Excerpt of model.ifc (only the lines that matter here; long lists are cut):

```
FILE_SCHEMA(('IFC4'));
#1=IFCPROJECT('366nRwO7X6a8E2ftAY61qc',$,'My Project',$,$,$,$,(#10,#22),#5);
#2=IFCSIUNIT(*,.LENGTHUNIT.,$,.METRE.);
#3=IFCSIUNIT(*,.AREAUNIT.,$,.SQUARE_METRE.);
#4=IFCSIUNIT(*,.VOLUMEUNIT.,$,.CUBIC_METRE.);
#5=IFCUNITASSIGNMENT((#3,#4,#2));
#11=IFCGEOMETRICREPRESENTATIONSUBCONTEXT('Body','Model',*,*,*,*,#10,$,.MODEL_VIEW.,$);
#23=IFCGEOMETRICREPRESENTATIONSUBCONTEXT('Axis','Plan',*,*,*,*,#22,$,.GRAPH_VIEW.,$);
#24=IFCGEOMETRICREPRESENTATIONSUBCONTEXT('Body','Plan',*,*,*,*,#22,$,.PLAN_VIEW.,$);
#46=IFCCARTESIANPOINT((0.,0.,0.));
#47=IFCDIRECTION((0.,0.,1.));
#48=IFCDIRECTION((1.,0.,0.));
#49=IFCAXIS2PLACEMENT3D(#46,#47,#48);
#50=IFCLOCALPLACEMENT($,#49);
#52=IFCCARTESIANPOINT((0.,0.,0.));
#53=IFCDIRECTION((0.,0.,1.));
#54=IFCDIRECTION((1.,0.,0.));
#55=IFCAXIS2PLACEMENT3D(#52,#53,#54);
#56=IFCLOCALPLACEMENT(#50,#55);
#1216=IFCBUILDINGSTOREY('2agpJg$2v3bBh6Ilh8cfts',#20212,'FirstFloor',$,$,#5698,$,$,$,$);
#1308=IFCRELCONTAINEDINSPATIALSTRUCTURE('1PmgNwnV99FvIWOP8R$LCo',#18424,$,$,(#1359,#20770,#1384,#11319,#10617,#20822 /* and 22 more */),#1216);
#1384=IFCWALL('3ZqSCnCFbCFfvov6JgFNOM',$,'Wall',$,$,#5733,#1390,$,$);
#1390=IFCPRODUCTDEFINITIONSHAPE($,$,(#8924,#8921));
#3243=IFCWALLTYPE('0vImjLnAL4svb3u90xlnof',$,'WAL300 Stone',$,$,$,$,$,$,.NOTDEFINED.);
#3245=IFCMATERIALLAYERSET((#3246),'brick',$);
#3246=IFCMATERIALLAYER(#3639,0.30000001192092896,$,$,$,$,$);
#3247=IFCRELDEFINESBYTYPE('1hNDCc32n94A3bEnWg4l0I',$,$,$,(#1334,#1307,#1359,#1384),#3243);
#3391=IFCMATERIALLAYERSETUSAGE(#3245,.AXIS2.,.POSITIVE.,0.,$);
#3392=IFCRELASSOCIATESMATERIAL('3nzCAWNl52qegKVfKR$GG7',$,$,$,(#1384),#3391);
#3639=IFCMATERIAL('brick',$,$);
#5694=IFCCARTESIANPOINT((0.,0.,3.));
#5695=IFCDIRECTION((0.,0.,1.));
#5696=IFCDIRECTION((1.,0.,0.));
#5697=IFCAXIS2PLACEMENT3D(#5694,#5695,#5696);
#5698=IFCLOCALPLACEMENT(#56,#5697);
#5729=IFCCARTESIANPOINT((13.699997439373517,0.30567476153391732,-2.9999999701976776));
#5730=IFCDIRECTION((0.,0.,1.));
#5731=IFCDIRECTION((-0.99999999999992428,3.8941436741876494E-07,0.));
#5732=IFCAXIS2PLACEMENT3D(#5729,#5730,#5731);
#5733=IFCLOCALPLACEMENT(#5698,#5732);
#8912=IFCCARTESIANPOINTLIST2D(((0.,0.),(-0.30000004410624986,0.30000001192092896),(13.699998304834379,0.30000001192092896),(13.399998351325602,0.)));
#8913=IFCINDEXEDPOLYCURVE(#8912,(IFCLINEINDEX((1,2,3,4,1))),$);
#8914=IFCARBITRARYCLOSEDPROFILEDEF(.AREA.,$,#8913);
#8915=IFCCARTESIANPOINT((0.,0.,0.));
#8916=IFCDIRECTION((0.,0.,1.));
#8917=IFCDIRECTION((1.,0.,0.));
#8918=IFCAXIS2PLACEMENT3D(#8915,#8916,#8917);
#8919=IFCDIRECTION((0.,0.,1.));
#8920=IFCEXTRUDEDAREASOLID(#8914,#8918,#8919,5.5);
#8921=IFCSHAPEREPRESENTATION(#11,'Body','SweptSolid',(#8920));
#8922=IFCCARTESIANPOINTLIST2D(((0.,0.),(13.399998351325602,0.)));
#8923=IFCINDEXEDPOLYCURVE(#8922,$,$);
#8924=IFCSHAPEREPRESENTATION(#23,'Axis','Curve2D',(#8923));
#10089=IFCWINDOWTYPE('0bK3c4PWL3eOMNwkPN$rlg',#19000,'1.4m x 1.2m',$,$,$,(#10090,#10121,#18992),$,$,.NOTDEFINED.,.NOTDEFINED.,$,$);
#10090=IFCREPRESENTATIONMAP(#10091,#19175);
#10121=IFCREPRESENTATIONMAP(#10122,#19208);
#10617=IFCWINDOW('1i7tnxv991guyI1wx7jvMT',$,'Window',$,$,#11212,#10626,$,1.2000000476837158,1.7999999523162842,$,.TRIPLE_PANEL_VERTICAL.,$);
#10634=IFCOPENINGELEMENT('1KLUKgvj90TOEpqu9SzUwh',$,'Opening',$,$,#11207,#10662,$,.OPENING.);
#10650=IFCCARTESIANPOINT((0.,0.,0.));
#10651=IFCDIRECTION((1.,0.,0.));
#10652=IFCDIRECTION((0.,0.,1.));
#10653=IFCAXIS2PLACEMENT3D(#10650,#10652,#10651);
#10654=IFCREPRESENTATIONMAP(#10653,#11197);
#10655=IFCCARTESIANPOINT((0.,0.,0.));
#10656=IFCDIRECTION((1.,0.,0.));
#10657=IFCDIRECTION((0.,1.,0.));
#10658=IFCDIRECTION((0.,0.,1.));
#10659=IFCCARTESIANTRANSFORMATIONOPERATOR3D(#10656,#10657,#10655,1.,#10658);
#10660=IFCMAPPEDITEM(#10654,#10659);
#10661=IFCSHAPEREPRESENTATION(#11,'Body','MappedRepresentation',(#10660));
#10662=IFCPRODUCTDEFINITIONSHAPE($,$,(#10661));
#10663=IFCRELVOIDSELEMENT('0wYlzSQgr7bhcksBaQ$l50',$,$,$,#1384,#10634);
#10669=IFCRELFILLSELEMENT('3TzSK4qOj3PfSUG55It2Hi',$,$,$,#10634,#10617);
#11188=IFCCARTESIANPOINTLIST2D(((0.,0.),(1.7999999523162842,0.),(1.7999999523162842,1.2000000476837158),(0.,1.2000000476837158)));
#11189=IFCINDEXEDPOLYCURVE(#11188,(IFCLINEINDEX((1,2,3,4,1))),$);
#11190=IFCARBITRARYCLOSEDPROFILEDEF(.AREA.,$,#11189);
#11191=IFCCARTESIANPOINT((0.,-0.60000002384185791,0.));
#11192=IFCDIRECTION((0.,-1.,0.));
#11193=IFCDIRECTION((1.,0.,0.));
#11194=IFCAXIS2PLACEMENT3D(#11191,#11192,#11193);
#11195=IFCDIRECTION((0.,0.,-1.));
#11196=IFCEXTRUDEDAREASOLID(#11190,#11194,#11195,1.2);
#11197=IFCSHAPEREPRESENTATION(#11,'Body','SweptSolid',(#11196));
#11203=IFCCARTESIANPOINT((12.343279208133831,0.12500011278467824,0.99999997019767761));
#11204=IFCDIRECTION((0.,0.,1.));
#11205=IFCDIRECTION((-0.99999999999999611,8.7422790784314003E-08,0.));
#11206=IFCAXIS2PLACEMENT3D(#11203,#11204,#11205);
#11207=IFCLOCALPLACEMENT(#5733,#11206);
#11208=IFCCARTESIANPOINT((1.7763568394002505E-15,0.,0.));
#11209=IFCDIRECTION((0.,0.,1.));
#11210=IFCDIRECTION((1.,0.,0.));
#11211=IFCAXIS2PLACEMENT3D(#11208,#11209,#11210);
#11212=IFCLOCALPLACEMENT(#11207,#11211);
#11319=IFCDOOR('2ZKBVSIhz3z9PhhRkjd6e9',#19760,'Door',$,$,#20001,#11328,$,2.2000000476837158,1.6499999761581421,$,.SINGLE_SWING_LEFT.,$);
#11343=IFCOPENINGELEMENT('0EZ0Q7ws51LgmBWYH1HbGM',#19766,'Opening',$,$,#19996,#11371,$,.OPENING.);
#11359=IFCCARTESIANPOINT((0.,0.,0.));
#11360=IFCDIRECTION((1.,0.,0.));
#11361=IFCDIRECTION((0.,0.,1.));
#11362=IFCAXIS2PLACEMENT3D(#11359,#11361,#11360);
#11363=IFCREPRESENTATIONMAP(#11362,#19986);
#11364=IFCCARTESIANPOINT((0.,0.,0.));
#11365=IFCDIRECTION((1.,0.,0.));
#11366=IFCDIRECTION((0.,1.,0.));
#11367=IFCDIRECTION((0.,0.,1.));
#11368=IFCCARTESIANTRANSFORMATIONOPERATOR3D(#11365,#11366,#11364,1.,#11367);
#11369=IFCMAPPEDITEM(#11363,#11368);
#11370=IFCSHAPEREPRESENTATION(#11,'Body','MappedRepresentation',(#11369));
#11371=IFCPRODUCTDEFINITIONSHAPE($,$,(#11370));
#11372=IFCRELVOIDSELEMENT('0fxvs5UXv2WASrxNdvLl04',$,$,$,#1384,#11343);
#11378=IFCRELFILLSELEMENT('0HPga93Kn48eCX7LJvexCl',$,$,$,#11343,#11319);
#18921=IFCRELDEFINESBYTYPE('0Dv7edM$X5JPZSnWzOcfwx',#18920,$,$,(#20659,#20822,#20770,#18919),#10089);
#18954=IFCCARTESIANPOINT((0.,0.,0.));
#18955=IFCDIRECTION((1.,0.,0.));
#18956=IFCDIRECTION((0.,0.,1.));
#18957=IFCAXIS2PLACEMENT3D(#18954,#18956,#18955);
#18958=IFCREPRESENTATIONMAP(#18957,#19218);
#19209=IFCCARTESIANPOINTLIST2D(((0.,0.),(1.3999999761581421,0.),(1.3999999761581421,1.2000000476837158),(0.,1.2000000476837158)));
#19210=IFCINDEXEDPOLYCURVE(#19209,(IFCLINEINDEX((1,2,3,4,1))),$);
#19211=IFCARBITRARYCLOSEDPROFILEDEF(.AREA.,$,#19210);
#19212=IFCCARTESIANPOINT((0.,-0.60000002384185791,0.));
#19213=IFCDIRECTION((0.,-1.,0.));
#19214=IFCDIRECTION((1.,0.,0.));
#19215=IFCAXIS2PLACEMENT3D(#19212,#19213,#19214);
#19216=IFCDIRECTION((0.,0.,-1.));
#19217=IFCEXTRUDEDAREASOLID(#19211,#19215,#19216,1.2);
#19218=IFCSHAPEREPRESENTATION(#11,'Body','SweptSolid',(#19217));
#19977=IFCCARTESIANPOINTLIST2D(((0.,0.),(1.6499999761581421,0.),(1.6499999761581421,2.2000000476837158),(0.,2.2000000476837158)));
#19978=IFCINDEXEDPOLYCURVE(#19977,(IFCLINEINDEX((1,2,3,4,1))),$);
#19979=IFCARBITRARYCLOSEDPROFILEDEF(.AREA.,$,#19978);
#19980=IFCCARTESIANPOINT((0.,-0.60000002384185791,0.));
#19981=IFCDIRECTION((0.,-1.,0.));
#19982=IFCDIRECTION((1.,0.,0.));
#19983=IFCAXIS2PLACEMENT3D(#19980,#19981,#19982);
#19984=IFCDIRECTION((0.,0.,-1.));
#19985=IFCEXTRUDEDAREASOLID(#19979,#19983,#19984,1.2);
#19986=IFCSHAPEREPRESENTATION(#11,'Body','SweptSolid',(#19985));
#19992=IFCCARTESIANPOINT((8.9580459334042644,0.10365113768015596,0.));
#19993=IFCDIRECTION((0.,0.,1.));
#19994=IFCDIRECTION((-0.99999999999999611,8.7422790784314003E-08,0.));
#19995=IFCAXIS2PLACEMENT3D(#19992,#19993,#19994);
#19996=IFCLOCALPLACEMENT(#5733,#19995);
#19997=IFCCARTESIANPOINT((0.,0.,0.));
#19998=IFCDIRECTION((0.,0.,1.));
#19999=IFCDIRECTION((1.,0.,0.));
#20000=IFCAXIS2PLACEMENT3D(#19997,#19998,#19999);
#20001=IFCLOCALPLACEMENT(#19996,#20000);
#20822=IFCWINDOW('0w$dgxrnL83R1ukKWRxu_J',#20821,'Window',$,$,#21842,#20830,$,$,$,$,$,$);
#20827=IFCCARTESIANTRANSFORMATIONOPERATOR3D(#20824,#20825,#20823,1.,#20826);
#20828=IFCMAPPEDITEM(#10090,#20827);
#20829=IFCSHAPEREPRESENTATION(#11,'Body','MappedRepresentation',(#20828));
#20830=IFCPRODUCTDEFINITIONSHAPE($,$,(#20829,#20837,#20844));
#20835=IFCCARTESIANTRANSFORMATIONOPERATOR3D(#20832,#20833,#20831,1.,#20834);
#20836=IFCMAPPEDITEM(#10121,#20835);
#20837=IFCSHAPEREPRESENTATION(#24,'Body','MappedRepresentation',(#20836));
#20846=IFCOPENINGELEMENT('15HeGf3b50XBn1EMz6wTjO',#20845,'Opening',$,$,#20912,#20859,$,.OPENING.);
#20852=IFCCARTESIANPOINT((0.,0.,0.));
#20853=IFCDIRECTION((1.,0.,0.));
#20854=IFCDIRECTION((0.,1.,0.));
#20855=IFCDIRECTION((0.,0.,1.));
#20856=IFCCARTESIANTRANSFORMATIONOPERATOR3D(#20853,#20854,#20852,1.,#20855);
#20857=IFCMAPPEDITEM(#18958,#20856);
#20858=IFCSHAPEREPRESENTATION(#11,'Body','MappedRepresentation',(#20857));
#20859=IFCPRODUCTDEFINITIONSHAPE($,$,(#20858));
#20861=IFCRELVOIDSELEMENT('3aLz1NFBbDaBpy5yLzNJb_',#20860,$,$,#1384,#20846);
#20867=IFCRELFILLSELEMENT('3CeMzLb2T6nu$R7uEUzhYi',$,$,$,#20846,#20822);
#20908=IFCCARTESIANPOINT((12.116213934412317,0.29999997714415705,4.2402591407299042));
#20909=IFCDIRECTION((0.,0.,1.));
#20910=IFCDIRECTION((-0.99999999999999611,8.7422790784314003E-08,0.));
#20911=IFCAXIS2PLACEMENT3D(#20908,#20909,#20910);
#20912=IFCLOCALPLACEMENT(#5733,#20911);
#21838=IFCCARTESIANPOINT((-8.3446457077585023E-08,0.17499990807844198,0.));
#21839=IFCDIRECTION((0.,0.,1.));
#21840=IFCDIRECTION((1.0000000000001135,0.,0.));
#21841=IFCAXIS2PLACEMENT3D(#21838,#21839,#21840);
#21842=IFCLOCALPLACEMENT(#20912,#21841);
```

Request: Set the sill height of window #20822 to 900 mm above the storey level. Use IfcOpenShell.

```python
import numpy as np
import ifcopenshell
import ifcopenshell.api.geometry
import ifcopenshell.geom
import ifcopenshell.util.element
import ifcopenshell.util.placement
import ifcopenshell.util.shape
import ifcopenshell.util.unit

model = ifcopenshell.open("model.ifc")
unit_scale = ifcopenshell.util.unit.calculate_unit_scale(model)

window = model.by_guid("0w$dgxrnL83R1ukKWRxu_J")
opening = window.FillsVoids[0].RelatingOpeningElement
storey = ifcopenshell.util.element.get_container(window, ifc_class="IfcBuildingStorey")
level = ifcopenshell.util.placement.get_local_placement(storey.ObjectPlacement)[2, 3]

# The opening's origin need not be at the sill, so measure its lowest point.
shape = ifcopenshell.geom.create_shape(ifcopenshell.geom.settings(), opening)
bottom = ifcopenshell.util.shape.get_shape_bottom_elevation(shape, shape.geometry) / unit_scale
dz = level + 0.9 - bottom

shift = np.array([0.0, 0.0, dz])
# The window is placed relative to its opening, so it follows when the opening moves.
matrix = ifcopenshell.util.placement.get_local_placement(opening.ObjectPlacement)
matrix[:3, 3] += shift
ifcopenshell.api.geometry.edit_object_placement(
    model, product=opening, matrix=matrix, is_si=False, should_transform_children=True
)

print(f"moved by {dz * unit_scale:+.3f} m")

model.write("model_edited.ifc")
```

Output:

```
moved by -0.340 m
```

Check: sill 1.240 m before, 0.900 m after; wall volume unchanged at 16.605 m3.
